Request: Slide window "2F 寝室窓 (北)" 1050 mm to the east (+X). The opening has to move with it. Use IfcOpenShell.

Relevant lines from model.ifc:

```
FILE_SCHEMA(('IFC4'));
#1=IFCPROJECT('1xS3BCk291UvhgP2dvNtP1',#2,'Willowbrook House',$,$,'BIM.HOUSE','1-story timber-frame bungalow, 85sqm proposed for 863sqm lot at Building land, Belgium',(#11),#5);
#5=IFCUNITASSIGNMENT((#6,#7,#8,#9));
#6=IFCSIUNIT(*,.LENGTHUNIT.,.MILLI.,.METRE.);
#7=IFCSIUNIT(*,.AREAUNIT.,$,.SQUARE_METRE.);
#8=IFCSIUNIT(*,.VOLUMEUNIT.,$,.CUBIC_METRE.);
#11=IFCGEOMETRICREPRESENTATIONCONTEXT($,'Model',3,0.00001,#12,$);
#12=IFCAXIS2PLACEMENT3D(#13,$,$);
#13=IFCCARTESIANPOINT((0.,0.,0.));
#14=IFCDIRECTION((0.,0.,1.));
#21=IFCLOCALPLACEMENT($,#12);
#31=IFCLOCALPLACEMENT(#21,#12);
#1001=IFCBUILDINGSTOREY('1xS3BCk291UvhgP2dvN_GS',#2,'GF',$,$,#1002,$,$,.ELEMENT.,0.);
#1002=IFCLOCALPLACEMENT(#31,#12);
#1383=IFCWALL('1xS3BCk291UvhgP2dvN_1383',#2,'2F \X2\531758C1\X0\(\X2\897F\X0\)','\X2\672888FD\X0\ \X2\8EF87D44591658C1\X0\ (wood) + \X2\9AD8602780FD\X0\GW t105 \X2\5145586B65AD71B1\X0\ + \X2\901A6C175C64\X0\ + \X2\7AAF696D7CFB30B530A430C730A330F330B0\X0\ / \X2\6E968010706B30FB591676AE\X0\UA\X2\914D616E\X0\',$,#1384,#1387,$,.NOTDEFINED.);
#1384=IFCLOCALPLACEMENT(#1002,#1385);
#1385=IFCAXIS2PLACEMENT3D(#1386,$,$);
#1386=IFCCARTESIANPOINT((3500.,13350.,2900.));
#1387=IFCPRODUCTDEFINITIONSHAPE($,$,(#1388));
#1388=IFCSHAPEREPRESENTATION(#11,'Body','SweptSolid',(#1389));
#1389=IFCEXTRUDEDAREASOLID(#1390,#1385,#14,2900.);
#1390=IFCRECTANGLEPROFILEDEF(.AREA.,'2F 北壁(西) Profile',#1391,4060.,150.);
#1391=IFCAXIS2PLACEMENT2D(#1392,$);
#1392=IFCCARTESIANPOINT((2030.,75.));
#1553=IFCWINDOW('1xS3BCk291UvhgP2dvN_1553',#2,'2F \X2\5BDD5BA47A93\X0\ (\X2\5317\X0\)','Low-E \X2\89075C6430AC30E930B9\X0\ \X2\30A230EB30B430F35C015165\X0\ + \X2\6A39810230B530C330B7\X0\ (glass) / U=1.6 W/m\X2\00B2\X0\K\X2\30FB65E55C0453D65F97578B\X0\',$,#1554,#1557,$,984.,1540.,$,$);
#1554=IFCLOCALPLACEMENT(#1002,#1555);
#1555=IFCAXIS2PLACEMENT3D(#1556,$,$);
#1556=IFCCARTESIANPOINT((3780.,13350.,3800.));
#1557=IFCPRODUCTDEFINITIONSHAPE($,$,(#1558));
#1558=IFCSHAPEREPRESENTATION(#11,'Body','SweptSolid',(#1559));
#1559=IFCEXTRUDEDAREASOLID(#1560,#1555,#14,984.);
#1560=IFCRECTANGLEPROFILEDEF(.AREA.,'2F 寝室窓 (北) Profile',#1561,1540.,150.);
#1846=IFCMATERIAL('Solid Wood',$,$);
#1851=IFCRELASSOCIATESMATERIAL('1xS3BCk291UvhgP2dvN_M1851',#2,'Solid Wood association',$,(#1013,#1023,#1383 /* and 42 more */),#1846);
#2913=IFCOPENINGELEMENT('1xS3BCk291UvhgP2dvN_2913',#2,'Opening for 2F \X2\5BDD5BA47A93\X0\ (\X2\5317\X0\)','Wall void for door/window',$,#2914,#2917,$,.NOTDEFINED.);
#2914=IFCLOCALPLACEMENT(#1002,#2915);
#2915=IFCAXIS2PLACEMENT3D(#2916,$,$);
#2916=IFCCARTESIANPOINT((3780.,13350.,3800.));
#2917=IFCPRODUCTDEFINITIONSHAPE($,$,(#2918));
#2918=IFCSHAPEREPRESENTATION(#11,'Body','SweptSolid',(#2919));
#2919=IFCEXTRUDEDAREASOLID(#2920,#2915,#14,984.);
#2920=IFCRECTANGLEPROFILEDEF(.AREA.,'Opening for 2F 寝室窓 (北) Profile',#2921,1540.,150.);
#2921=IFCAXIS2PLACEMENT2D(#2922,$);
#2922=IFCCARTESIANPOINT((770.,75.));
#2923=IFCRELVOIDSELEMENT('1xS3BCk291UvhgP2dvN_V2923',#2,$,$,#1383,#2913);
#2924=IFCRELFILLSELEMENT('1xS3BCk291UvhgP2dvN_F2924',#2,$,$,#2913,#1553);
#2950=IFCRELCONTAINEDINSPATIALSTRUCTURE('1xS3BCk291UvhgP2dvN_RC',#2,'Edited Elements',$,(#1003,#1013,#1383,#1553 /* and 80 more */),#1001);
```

```python
import ifcopenshell
import ifcopenshell.api.geometry
import ifcopenshell.util.placement

model = ifcopenshell.open("model.ifc")

window = model.by_guid("1xS3BCk291UvhgP2dvN_1553")
opening = window.FillsVoids[0].RelatingOpeningElement
wall = opening.VoidsElements[0].RelatingBuildingElement

wall_matrix = ifcopenshell.util.placement.get_local_placement(wall.ObjectPlacement)
shift = wall_matrix[:3, 0] * 1050.0
before = ifcopenshell.util.placement.get_local_placement(window.ObjectPlacement)[:3, 3].copy()

# The window is not placed relative to its opening, so move both.
for product in (opening, window):
    matrix = ifcopenshell.util.placement.get_local_placement(product.ObjectPlacement)
    matrix[:3, 3] += shift
    ifcopenshell.api.geometry.edit_object_placement(model, product=product, matrix=matrix, is_si=False)

after = ifcopenshell.util.placement.get_local_placement(window.ObjectPlacement)[:3, 3]
print("window moved by", (after - before).round(3) + 0.0)

model.write("model_v2.ifc")
```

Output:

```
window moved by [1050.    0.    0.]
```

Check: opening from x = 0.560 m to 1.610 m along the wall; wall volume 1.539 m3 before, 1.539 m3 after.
